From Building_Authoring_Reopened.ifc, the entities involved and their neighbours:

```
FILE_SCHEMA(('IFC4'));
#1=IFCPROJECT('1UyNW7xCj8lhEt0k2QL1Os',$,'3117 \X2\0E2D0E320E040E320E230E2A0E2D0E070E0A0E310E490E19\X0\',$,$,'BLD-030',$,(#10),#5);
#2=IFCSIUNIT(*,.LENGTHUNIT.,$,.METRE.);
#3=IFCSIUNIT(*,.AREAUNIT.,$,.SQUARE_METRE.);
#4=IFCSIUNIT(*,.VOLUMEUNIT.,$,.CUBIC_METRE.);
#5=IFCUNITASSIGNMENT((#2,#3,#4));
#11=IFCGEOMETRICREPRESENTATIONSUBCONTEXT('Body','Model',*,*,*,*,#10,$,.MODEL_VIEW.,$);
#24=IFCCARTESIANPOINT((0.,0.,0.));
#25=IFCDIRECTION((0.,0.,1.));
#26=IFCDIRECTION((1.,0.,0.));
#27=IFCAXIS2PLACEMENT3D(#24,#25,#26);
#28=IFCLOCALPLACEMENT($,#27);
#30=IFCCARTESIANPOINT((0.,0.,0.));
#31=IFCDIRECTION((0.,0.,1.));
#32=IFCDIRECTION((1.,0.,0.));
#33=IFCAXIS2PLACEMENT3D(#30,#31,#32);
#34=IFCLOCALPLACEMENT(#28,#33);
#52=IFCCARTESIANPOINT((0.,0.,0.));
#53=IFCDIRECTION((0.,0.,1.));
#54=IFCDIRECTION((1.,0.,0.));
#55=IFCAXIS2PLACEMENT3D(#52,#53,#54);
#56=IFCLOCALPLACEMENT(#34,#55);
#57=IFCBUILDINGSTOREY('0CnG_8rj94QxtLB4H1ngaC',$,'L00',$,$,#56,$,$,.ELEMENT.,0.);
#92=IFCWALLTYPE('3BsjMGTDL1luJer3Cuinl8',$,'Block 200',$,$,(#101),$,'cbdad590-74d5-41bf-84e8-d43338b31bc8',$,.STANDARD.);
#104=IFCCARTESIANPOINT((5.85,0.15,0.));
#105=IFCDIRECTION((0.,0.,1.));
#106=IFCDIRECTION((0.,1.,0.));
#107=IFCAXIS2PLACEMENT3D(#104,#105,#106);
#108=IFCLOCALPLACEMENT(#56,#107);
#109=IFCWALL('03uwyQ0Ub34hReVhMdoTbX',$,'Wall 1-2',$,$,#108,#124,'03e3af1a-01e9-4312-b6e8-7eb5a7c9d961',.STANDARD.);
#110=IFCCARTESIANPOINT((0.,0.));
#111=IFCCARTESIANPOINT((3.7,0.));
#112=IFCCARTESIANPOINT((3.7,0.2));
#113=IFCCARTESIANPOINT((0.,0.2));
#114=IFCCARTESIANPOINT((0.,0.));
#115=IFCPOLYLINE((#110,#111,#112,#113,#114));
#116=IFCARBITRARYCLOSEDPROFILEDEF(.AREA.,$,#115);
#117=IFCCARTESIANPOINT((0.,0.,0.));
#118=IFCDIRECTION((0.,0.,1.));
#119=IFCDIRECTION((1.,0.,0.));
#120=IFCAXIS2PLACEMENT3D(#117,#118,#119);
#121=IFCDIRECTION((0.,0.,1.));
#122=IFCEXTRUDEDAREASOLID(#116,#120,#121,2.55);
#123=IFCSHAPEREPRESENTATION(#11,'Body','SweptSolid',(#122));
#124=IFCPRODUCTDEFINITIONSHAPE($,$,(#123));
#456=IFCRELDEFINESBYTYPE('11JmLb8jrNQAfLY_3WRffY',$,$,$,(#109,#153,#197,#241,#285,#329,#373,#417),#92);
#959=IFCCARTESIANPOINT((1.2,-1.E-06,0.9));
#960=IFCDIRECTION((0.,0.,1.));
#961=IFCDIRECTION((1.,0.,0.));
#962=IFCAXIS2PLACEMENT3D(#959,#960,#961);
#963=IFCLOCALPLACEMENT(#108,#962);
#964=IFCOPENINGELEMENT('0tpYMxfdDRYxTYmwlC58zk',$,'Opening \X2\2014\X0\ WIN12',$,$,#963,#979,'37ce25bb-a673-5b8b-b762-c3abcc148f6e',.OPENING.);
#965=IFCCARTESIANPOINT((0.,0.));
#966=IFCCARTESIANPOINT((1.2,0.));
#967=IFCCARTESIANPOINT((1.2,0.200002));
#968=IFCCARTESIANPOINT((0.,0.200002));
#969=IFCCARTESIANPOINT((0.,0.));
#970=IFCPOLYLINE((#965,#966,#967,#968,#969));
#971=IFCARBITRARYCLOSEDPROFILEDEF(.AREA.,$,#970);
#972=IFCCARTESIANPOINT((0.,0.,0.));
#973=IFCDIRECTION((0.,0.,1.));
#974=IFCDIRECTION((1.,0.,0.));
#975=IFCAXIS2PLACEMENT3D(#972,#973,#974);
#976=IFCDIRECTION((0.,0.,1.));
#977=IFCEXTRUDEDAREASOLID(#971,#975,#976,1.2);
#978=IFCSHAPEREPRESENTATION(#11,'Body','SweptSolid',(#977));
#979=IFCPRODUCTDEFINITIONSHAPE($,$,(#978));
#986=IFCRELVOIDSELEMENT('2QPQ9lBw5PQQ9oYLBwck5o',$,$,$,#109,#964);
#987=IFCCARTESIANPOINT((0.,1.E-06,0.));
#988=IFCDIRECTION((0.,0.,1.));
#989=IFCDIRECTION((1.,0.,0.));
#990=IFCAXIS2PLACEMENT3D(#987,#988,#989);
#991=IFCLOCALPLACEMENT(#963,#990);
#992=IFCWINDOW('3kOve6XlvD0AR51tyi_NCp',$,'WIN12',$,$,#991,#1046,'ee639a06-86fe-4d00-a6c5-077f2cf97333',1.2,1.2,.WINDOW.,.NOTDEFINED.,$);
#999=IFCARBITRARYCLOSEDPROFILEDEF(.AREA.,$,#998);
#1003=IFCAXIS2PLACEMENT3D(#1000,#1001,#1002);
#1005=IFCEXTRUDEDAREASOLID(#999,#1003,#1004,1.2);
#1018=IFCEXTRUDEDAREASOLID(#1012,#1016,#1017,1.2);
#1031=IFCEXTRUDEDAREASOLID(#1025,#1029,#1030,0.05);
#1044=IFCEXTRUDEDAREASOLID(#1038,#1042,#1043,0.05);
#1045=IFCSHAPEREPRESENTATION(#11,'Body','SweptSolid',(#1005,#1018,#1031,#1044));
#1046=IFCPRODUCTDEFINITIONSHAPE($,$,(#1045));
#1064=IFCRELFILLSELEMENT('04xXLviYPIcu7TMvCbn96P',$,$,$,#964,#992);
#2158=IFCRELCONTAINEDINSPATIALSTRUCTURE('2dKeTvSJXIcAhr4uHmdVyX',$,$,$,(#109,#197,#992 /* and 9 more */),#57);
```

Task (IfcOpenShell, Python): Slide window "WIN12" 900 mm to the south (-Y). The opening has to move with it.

```python
import ifcopenshell
import ifcopenshell.api.geometry
import ifcopenshell.util.placement
import ifcopenshell.util.unit

model = ifcopenshell.open("Building_Authoring_Reopened.ifc")
unit_scale = ifcopenshell.util.unit.calculate_unit_scale(model)

window = model.by_guid("3kOve6XlvD0AR51tyi_NCp")
opening = window.FillsVoids[0].RelatingOpeningElement
wall = opening.VoidsElements[0].RelatingBuildingElement

wall_matrix = ifcopenshell.util.placement.get_local_placement(wall.ObjectPlacement)
shift = wall_matrix[:3, 0] * -0.9 / unit_scale
before = ifcopenshell.util.placement.get_local_placement(window.ObjectPlacement)[:3, 3].copy()

# The window is placed relative to its opening, so it follows when the opening moves.
matrix = ifcopenshell.util.placement.get_local_placement(opening.ObjectPlacement)
matrix[:3, 3] += shift
ifcopenshell.api.geometry.edit_object_placement(
    model, product=opening, matrix=matrix, is_si=False, should_transform_children=True
)

after = ifcopenshell.util.placement.get_local_placement(window.ObjectPlacement)[:3, 3]
print("window moved by", (after - before).round(3) + 0.0)

model.write("Building_Authoring_Reopened_v2.ifc")
```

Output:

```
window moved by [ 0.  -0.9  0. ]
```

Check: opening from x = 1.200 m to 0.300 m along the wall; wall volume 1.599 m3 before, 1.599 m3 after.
